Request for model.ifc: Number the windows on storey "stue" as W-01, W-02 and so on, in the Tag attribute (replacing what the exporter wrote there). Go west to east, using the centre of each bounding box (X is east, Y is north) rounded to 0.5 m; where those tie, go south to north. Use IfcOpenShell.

First a look at what the model holds.

```python
import ifcopenshell
import ifcopenshell.util.element
import ifcopenshell.util.placement

model = ifcopenshell.open("model.ifc")
print(model.schema)
storey = next(s for s in model.by_type("IfcBuildingStorey") if s.Name == "stue")
windows = [e for e in ifcopenshell.util.element.get_decomposition(storey) if e.is_a("IfcWindow")]
for e in sorted(windows, key=lambda e: e.id()):
    origin = ifcopenshell.util.placement.get_local_placement(e.ObjectPlacement)[:3, 3]
    print(e.id(), e.Tag, e.Name, origin.round(2) + 0.0, sep=" | ")
```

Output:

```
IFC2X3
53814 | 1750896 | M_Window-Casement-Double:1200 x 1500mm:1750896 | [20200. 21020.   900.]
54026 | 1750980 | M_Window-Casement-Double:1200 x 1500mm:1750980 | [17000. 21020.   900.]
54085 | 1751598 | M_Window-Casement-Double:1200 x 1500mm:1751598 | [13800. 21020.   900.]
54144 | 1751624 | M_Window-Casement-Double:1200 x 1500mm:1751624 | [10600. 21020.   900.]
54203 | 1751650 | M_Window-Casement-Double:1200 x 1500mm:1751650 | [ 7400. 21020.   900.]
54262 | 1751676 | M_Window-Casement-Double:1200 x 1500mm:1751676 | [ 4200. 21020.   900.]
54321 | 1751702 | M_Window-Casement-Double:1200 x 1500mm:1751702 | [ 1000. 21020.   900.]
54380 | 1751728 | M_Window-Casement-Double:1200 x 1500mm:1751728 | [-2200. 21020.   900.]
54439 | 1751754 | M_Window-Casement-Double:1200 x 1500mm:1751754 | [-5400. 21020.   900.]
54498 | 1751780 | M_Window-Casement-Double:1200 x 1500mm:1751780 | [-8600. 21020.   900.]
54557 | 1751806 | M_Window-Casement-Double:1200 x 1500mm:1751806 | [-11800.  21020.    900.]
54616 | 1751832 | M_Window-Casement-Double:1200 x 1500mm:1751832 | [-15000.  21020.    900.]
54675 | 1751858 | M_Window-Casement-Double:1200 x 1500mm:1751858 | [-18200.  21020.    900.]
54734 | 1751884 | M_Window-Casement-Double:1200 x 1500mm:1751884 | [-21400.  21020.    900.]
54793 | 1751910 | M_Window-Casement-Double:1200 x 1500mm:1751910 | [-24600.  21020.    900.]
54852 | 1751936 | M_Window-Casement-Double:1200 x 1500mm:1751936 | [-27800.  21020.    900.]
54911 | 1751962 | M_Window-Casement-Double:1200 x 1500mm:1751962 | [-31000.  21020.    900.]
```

```python
import ifcopenshell
import ifcopenshell.geom
import ifcopenshell.util.element
import ifcopenshell.util.shape

model = ifcopenshell.open("model.ifc")
settings = ifcopenshell.geom.settings()
settings.set("use-world-coords", True)


def centre(element):
    shape = ifcopenshell.geom.create_shape(settings, element)
    return ifcopenshell.util.shape.get_bbox_centroid(shape.geometry)


storey = next(s for s in model.by_type("IfcBuildingStorey") if s.Name == "stue")
windows = [e for e in ifcopenshell.util.element.get_decomposition(storey) if e.is_a("IfcWindow")]

# Insertion points can sit at a corner or the storey origin, so sort by the geometry (in metres).
centres = {e: centre(e) for e in windows}
windows.sort(key=lambda e: (round(centres[e][0] / 0.5), centres[e][1]))

for i, e in enumerate(windows, start=1):
    number = f"W-{i:02d}"
    e.Tag = number
    print(e.id(), number)

model.write("model_updated.ifc")
```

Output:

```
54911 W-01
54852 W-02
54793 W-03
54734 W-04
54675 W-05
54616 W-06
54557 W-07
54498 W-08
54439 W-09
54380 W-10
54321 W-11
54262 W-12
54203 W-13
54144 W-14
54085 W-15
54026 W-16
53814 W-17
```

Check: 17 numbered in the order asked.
